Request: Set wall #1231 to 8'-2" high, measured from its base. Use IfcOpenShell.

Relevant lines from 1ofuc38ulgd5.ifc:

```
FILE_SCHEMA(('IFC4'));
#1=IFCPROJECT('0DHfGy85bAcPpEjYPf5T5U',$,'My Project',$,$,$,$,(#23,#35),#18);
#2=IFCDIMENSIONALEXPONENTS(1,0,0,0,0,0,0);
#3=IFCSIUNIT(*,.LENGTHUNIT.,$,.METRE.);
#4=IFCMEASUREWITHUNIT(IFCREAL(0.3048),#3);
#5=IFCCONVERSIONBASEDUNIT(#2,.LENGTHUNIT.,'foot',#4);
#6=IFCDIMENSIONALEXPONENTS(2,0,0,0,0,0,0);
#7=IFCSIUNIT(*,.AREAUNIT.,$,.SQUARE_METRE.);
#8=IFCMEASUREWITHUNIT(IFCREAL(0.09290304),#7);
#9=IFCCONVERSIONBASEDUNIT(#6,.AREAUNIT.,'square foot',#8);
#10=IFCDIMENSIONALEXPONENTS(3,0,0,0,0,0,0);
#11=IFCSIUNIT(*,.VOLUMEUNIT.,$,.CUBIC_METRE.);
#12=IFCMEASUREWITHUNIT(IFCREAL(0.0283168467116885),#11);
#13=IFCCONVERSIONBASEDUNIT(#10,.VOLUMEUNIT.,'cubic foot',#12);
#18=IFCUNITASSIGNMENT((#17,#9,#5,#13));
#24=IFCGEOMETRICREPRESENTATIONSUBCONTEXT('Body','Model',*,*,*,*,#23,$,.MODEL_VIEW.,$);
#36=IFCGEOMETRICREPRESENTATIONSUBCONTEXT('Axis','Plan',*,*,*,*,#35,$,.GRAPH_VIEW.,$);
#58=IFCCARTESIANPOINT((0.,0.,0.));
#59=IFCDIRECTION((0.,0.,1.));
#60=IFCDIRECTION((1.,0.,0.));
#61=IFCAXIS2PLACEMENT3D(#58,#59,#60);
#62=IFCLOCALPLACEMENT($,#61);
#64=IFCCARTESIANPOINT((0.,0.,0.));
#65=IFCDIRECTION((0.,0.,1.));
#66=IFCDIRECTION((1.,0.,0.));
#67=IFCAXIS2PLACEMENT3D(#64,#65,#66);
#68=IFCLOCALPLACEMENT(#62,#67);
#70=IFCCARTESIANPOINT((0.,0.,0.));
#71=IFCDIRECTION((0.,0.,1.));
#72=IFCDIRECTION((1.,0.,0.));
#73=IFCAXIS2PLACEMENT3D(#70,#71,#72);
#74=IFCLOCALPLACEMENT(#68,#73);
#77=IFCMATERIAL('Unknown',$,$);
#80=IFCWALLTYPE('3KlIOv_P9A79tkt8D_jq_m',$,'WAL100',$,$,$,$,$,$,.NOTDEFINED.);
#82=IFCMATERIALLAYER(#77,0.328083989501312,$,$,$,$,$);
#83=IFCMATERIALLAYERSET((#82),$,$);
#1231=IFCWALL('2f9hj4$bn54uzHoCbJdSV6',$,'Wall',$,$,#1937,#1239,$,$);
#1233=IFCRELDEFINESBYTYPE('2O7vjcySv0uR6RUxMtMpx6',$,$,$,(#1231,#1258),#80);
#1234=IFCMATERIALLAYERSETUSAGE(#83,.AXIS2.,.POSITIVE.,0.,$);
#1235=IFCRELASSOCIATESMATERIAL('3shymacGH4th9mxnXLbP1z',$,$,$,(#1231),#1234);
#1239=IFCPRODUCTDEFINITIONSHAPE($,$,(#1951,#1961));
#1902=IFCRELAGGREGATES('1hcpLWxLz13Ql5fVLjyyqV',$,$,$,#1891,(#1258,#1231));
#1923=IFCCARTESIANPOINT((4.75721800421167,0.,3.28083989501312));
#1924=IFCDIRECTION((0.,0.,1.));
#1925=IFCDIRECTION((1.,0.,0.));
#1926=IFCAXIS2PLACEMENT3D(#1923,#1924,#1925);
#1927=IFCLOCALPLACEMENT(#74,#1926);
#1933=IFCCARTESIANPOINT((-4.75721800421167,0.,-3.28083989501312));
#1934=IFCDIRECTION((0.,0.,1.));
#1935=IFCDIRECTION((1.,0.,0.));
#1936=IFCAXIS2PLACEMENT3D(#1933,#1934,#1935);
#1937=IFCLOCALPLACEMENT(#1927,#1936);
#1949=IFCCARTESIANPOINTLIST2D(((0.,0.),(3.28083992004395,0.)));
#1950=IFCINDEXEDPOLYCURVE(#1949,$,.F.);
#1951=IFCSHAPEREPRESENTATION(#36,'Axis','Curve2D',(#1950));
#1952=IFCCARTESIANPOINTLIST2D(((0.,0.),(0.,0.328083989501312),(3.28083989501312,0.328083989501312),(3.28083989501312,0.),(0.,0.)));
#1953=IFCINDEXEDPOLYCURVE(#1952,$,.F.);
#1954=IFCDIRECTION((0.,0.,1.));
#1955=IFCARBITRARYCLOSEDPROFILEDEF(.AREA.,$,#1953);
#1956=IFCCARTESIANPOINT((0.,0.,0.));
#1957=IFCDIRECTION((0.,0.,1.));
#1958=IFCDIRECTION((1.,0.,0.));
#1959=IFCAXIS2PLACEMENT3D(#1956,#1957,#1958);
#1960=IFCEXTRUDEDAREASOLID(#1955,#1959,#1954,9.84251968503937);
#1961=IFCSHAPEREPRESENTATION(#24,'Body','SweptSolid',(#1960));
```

```python
import ifcopenshell
import ifcopenshell.geom
import ifcopenshell.util.representation
import ifcopenshell.util.shape
import ifcopenshell.util.unit

model = ifcopenshell.open("1ofuc38ulgd5.ifc")
unit_scale = ifcopenshell.util.unit.calculate_unit_scale(model)
settings = ifcopenshell.geom.settings()


def volume(element):
    """Net volume in cubic metres, openings subtracted."""
    shape = ifcopenshell.geom.create_shape(settings, element)
    return ifcopenshell.util.shape.get_volume(shape.geometry)


wall = model.by_id(1231)
before = volume(wall)

body = ifcopenshell.util.representation.get_representation(wall, "Model", "Body")
solid = body.Items[0]
old_height = solid.Depth
solid.Depth = 98 * 0.0254 / unit_scale
after = volume(wall)

print(f"height {old_height:g} -> {solid.Depth:g}, volume {before:.3f} -> {after:.3f} m3")

model.write("1ofuc38ulgd5_v2.ifc")
```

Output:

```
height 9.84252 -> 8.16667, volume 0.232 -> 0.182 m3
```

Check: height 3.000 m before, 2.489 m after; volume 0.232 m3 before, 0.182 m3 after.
